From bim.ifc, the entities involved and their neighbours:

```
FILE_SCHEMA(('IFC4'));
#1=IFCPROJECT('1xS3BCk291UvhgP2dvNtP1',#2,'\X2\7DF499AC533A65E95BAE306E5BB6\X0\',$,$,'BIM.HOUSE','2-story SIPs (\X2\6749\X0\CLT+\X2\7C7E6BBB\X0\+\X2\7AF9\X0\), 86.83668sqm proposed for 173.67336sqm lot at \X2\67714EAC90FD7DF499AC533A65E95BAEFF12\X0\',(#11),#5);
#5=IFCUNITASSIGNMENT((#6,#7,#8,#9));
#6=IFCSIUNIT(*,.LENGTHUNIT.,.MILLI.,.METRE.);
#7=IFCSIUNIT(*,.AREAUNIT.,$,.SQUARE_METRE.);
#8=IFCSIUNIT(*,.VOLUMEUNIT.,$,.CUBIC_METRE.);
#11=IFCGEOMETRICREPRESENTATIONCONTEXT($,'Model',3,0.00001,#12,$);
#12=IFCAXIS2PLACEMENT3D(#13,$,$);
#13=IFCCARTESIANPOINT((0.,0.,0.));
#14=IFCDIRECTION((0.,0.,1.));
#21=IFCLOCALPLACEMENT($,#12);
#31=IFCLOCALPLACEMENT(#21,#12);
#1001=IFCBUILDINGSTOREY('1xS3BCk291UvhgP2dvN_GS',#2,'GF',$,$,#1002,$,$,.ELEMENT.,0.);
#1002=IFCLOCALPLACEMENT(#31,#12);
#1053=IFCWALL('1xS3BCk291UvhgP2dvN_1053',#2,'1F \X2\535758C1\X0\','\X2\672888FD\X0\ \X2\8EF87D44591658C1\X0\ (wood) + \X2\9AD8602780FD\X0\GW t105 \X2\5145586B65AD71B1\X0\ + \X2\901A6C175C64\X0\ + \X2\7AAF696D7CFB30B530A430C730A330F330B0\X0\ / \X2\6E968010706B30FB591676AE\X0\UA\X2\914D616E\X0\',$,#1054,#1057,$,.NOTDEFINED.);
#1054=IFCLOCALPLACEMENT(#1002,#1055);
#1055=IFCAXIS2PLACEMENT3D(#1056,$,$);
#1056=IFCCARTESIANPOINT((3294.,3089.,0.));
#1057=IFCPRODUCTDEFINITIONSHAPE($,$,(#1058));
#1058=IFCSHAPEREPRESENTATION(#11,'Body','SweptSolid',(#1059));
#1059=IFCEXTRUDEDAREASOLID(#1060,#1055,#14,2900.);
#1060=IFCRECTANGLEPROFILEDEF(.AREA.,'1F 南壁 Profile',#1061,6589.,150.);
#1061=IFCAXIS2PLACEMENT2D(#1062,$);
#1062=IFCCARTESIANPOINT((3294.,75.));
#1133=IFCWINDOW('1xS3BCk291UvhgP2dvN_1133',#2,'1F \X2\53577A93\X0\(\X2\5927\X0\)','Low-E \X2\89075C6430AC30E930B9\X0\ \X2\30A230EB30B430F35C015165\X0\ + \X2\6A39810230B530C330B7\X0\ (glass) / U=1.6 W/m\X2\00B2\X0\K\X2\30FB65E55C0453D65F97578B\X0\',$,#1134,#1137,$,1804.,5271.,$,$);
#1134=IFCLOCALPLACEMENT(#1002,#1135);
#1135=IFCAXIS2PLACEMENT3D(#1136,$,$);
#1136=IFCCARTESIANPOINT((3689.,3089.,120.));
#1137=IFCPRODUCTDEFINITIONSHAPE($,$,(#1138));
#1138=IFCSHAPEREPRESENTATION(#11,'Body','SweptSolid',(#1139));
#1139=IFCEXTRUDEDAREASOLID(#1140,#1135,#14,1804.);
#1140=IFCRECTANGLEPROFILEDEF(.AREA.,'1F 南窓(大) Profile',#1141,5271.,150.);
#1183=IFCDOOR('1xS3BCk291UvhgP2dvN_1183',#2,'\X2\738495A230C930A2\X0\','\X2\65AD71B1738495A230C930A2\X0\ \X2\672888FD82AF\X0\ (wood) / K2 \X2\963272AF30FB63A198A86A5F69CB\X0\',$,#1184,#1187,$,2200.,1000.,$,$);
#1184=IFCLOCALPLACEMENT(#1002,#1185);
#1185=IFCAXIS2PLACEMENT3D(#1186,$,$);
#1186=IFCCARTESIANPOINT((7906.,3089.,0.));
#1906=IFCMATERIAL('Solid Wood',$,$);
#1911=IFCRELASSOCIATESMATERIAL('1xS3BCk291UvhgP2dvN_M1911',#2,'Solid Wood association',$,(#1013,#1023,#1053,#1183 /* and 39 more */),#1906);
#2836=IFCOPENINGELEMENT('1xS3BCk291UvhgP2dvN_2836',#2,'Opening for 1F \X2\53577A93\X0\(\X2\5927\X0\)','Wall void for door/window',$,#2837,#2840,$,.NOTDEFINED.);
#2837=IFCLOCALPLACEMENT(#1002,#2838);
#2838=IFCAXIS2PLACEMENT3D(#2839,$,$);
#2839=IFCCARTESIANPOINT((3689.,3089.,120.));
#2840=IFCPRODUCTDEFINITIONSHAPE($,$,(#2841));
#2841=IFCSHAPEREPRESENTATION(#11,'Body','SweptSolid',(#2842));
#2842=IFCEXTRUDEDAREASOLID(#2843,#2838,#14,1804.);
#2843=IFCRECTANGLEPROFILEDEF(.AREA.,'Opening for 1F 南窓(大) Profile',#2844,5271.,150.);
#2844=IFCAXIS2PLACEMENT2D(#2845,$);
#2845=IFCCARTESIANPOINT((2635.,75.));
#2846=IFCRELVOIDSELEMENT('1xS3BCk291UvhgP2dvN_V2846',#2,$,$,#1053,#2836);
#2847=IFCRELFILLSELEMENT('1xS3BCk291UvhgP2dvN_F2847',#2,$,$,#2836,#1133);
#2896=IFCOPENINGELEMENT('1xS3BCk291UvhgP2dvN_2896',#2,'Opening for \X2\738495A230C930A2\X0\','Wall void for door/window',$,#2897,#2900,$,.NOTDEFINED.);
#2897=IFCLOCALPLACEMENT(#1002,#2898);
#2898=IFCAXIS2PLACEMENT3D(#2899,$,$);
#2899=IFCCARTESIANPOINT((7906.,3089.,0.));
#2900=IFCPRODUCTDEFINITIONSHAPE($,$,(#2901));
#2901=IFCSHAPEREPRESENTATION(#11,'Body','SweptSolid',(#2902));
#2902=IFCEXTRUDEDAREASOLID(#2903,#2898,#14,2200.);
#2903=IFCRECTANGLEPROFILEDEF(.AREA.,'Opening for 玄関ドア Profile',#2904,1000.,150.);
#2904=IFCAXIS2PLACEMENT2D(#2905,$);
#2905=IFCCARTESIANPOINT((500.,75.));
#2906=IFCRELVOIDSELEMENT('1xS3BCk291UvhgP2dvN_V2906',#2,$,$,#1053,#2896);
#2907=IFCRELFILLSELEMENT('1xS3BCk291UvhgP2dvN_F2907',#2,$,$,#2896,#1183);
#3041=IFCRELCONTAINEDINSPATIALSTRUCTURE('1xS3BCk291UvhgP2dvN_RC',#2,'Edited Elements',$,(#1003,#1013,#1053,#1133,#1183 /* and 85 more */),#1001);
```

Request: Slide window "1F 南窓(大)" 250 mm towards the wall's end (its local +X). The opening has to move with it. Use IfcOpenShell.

```python
import ifcopenshell
import ifcopenshell.api.geometry
import ifcopenshell.util.placement
import ifcopenshell.util.unit

model = ifcopenshell.open("bim.ifc")
unit_scale = ifcopenshell.util.unit.calculate_unit_scale(model)

window = model.by_guid("1xS3BCk291UvhgP2dvN_1133")
opening = window.FillsVoids[0].RelatingOpeningElement
wall = opening.VoidsElements[0].RelatingBuildingElement

wall_matrix = ifcopenshell.util.placement.get_local_placement(wall.ObjectPlacement)
shift = wall_matrix[:3, 0] * 0.25 / unit_scale
before = ifcopenshell.util.placement.get_local_placement(window.ObjectPlacement)[:3, 3].copy()

# The window is not placed relative to its opening, so move both.
for product in (opening, window):
    matrix = ifcopenshell.util.placement.get_local_placement(product.ObjectPlacement)
    matrix[:3, 3] += shift
    ifcopenshell.api.geometry.edit_object_placement(model, product=product, matrix=matrix, is_si=False)

after = ifcopenshell.util.placement.get_local_placement(window.ObjectPlacement)[:3, 3]
print("window moved by", (after - before).round(3) + 0.0)

model.write("bim_updated.ifc")
```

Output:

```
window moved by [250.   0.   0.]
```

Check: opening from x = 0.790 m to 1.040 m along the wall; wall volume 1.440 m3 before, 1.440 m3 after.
